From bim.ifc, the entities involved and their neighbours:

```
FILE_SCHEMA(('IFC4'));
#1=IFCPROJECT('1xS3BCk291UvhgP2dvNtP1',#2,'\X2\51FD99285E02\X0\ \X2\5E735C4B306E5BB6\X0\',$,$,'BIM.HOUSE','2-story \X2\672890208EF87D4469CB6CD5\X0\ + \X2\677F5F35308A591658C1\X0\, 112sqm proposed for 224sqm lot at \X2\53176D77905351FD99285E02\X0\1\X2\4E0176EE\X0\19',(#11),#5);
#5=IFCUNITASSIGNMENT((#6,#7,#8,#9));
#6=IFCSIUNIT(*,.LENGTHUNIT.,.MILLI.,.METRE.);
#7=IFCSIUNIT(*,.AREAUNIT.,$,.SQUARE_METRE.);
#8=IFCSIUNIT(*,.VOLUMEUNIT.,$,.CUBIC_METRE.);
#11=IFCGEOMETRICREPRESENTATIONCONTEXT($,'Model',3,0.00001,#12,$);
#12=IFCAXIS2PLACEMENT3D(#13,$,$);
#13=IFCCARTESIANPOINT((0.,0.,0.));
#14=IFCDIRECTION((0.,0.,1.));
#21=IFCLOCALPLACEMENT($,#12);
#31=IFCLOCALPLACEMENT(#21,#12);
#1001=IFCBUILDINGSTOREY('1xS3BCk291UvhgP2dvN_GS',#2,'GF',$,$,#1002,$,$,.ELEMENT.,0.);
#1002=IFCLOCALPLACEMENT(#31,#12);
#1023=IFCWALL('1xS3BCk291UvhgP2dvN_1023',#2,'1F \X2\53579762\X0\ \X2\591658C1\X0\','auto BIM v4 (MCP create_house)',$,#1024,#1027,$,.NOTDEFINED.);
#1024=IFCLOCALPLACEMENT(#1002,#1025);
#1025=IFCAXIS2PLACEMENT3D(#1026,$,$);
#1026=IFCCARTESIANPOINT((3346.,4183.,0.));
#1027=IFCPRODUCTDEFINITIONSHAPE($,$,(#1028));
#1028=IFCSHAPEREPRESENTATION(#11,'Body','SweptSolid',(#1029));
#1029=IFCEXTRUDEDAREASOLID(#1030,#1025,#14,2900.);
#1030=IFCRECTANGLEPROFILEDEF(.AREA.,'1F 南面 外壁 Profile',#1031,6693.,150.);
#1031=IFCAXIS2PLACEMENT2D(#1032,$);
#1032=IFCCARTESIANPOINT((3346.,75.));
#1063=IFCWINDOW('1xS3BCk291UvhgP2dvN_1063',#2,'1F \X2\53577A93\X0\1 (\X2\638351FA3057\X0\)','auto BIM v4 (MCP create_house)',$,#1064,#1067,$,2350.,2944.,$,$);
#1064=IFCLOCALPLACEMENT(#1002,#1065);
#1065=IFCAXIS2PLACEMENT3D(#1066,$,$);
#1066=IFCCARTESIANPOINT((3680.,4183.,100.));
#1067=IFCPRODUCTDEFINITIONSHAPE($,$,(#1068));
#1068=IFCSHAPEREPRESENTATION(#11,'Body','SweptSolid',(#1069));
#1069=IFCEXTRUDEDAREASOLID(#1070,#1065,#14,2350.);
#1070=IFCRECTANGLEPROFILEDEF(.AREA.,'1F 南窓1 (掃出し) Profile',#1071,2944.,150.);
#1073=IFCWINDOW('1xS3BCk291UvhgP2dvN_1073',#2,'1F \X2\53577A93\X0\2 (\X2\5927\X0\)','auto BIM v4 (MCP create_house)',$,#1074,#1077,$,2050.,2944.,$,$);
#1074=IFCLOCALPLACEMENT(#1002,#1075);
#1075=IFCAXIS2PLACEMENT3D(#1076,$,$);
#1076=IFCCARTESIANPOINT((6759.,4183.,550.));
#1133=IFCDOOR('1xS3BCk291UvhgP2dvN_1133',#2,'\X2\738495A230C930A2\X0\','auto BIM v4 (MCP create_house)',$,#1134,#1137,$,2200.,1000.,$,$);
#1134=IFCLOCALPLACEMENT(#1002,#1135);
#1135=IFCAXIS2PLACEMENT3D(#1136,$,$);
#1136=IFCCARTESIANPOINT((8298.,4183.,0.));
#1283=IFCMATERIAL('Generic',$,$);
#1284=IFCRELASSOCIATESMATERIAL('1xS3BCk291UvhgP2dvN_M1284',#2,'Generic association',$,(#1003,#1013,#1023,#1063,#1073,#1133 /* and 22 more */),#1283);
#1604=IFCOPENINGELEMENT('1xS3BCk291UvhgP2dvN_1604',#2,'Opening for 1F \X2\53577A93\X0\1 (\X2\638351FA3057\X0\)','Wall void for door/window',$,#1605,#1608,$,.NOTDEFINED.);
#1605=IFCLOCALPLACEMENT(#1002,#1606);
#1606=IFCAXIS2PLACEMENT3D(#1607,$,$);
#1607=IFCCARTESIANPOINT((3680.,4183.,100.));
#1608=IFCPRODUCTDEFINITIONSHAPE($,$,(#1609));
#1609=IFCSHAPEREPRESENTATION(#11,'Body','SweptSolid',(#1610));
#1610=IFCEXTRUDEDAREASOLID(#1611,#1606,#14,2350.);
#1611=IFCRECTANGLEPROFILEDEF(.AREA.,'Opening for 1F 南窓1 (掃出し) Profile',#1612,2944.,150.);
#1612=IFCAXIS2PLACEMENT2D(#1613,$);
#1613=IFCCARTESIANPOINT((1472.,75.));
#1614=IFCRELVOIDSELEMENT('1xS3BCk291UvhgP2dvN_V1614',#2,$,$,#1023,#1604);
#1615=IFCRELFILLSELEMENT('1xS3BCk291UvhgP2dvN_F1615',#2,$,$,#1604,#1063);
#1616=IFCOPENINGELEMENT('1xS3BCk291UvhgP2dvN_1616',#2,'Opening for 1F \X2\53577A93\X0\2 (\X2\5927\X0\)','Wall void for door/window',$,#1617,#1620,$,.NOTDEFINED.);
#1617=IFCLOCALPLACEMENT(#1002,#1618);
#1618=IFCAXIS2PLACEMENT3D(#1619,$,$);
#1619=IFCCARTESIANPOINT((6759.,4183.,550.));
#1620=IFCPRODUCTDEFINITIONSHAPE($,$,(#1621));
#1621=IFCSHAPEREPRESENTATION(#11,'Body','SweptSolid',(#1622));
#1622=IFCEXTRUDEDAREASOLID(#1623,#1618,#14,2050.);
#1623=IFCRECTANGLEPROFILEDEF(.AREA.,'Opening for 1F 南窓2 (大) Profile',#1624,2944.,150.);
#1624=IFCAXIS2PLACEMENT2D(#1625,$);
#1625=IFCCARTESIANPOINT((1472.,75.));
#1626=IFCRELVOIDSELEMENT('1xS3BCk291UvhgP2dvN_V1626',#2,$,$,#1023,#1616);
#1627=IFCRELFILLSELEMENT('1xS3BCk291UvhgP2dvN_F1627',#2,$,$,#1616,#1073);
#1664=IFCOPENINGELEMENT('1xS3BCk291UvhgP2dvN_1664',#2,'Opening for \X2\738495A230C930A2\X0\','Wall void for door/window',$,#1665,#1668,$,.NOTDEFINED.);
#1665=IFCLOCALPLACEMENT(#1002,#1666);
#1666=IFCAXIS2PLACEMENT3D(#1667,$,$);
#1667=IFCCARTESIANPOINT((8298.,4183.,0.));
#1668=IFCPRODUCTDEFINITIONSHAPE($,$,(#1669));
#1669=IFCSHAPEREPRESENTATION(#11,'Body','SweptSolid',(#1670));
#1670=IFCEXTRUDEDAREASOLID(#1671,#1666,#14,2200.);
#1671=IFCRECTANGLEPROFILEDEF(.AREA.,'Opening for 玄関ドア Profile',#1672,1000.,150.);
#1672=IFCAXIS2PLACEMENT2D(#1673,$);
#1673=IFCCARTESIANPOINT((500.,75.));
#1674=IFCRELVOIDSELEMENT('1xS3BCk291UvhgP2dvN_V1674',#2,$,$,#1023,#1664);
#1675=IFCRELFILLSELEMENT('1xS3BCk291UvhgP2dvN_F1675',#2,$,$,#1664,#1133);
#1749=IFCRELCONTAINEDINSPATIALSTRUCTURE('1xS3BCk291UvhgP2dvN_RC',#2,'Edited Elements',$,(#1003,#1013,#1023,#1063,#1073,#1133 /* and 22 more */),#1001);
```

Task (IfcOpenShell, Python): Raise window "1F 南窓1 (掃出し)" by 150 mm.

```python
import numpy as np
import ifcopenshell
import ifcopenshell.api.geometry
import ifcopenshell.util.placement
import ifcopenshell.util.unit

model = ifcopenshell.open("bim.ifc")
unit_scale = ifcopenshell.util.unit.calculate_unit_scale(model)

window = model.by_guid("1xS3BCk291UvhgP2dvN_1063")
opening = window.FillsVoids[0].RelatingOpeningElement
dz = 150.0

shift = np.array([0.0, 0.0, dz])
# The window is not placed relative to its opening, so move both.
for product in (opening, window):
    matrix = ifcopenshell.util.placement.get_local_placement(product.ObjectPlacement)
    matrix[:3, 3] += shift
    ifcopenshell.api.geometry.edit_object_placement(model, product=product, matrix=matrix, is_si=False)

print(f"moved by {dz * unit_scale:+.3f} m")

model.write("bim_rev.ifc")
```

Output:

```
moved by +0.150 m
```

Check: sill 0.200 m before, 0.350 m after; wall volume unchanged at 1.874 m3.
